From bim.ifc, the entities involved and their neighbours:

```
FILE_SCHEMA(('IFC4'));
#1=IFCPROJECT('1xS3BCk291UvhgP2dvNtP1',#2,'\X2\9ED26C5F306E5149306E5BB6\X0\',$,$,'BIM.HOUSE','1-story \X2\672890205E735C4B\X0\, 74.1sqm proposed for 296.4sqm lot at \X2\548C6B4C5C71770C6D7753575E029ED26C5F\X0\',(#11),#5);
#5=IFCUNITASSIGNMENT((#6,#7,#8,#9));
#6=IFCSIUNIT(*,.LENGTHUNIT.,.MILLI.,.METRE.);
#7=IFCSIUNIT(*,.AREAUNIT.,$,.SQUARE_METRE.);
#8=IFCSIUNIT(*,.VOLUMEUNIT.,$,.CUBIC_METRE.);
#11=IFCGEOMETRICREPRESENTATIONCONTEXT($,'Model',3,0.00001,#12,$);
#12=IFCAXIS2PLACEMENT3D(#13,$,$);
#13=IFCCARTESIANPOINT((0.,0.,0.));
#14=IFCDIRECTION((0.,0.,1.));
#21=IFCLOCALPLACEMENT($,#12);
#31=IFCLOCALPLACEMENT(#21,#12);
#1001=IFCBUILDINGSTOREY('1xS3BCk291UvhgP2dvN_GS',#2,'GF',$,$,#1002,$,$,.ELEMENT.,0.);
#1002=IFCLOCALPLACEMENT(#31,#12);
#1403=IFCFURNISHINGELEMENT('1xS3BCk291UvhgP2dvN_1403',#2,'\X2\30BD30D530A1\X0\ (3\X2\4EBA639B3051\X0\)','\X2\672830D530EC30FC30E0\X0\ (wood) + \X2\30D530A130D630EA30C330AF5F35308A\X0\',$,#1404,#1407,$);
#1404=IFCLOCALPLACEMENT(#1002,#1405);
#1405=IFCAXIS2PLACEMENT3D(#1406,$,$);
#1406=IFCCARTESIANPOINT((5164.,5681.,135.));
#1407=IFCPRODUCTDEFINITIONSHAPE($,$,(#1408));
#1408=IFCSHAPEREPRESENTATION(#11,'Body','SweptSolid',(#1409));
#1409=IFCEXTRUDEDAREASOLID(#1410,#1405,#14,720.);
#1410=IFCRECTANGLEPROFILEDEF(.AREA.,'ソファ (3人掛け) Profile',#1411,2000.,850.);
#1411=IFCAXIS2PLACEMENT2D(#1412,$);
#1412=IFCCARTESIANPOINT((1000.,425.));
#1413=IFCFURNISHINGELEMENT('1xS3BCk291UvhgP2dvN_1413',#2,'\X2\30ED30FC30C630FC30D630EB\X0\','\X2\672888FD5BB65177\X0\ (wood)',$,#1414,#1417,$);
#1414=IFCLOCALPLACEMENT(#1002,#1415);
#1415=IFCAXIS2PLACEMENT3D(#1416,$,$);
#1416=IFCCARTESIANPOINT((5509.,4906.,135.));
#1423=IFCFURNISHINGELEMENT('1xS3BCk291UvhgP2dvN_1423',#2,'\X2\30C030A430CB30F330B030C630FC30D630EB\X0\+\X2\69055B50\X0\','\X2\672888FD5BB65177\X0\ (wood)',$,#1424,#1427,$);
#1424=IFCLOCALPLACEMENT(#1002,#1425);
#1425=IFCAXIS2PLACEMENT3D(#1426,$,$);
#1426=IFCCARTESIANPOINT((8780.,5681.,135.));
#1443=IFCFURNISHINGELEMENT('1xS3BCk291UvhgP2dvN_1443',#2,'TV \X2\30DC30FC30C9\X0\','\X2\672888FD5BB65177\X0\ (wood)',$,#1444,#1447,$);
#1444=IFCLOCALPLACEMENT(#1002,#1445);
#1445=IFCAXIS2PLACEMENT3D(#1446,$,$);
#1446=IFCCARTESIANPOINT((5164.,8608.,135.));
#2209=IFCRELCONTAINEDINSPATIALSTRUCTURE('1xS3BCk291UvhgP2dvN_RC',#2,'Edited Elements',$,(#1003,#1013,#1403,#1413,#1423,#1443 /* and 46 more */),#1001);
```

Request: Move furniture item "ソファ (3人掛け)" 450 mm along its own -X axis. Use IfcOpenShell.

```python
import ifcopenshell
import ifcopenshell.api.geometry
import ifcopenshell.util.placement
import ifcopenshell.util.unit

model = ifcopenshell.open("bim.ifc")
unit_scale = ifcopenshell.util.unit.calculate_unit_scale(model)

item = model.by_guid("1xS3BCk291UvhgP2dvN_1403")
matrix = ifcopenshell.util.placement.get_local_placement(item.ObjectPlacement)
matrix[:3, 3] -= matrix[:3, 0] * 0.45 / unit_scale
ifcopenshell.api.geometry.edit_object_placement(model, product=item, matrix=matrix, is_si=False)

print(ifcopenshell.util.placement.get_local_placement(item.ObjectPlacement).round(3) + 0.0)

model.write("bim_updated.ifc")
```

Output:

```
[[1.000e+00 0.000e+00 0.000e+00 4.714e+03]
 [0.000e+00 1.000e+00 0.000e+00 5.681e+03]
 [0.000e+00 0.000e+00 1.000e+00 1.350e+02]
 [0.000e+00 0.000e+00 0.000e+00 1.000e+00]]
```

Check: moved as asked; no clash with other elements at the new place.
